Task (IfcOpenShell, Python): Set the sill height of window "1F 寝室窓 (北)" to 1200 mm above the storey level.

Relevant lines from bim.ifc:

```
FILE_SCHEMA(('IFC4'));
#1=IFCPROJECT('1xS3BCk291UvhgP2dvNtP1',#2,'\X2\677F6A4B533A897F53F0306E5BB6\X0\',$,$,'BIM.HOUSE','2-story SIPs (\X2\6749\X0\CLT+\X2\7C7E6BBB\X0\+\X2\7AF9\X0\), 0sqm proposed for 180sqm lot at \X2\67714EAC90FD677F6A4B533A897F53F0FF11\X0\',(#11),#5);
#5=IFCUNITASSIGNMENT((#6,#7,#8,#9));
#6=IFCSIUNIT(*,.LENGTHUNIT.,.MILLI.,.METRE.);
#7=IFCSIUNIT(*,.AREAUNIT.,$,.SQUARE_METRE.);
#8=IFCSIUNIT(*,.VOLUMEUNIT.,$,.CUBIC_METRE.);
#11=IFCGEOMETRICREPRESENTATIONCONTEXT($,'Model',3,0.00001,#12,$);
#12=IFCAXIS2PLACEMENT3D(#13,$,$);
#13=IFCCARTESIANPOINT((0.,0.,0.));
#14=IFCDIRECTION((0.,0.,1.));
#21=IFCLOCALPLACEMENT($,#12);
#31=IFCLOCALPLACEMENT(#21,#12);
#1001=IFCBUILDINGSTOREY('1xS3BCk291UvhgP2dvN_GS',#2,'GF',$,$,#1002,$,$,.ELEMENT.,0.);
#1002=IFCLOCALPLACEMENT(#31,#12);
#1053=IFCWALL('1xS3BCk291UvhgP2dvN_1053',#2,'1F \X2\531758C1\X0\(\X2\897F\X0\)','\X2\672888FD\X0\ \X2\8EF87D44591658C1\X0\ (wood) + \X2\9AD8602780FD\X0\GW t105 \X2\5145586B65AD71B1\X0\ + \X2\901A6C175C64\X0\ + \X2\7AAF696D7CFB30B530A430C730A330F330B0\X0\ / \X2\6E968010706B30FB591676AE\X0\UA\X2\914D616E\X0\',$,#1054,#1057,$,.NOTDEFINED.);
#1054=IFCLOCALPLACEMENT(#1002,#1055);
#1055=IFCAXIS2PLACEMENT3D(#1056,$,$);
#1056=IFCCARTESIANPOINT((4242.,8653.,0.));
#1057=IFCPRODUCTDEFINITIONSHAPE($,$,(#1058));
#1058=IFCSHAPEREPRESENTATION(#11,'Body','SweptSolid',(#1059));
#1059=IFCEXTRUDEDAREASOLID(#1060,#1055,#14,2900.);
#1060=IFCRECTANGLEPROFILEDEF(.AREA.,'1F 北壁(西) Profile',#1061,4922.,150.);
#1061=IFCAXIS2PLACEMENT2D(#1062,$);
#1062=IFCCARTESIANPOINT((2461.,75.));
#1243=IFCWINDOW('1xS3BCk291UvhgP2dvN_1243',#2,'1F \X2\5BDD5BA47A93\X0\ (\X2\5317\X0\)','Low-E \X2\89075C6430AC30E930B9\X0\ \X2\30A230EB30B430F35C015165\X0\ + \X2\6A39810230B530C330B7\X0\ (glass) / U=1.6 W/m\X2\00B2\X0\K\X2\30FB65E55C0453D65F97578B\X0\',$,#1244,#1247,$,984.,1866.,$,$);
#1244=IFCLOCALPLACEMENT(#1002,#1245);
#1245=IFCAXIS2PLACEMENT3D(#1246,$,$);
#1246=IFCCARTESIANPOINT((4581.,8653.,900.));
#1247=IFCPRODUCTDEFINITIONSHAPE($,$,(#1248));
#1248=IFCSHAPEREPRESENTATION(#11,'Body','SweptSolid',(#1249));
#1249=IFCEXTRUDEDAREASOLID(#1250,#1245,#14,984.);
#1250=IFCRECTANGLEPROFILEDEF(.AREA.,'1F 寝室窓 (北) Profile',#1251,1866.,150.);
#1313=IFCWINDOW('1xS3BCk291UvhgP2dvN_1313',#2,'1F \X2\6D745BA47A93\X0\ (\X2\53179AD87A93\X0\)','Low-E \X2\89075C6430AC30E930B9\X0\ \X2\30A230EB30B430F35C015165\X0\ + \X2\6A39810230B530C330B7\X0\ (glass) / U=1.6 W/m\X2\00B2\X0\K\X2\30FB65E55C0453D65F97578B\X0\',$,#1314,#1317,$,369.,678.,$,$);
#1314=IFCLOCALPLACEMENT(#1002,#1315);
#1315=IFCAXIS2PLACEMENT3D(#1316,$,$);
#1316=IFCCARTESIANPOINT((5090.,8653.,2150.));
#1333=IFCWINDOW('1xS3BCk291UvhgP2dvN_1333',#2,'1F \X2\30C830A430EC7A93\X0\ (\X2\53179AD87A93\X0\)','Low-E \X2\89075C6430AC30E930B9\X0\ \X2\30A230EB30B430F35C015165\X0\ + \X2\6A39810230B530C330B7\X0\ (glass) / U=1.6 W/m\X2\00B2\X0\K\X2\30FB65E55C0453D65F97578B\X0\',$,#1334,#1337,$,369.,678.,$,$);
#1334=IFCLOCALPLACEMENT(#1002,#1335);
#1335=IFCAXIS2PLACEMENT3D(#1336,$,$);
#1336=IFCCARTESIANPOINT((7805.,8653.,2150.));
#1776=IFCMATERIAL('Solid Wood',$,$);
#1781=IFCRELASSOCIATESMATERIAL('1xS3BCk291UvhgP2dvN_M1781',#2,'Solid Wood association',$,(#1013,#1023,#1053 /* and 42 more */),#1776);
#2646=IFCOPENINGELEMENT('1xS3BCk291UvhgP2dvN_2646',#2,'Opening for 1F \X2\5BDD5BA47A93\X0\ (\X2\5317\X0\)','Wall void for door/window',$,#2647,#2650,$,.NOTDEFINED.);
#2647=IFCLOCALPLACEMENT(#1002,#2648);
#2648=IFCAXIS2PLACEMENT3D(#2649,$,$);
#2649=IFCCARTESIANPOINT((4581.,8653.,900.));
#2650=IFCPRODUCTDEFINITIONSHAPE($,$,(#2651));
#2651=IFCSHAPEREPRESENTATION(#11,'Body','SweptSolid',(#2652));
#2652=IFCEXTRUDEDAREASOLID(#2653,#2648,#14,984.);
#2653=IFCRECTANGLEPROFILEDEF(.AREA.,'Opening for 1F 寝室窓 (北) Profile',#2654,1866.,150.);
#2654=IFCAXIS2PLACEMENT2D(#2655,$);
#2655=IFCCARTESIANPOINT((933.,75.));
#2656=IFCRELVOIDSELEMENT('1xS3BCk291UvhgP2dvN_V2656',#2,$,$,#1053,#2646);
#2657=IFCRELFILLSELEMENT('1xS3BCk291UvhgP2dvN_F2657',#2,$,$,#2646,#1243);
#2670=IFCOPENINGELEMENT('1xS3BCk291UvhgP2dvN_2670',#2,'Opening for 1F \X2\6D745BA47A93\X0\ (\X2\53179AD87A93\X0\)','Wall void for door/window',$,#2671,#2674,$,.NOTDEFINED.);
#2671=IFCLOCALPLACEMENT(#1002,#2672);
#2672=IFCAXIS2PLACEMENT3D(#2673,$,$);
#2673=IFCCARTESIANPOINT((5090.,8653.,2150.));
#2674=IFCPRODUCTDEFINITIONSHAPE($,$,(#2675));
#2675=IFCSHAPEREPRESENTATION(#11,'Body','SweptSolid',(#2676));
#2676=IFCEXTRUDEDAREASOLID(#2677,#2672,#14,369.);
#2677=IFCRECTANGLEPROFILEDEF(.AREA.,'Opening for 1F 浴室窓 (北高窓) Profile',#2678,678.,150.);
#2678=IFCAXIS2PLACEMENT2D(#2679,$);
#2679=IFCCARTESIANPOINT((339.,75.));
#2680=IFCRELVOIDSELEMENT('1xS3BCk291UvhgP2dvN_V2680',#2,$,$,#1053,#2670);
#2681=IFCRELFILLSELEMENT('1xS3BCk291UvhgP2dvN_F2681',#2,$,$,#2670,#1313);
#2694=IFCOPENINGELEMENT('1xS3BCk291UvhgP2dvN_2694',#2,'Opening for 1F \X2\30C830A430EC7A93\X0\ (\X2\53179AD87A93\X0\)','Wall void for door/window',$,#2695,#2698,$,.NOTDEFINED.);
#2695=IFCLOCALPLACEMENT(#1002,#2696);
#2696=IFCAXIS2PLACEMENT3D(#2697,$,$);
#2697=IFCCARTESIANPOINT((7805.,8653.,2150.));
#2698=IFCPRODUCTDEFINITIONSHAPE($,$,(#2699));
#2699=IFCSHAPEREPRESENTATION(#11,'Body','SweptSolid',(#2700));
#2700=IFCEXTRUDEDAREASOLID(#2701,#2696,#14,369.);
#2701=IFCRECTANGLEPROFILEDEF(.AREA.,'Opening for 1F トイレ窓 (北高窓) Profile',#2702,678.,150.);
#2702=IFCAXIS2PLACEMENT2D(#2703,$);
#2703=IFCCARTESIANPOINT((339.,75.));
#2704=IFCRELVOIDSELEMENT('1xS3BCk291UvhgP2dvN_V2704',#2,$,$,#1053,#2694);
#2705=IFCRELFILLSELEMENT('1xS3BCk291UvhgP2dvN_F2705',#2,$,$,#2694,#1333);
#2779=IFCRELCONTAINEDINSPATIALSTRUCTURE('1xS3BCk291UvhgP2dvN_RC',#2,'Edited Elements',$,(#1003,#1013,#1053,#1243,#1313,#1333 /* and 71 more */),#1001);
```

```python
import numpy as np
import ifcopenshell
import ifcopenshell.api.geometry
import ifcopenshell.geom
import ifcopenshell.util.element
import ifcopenshell.util.placement
import ifcopenshell.util.shape
import ifcopenshell.util.unit

model = ifcopenshell.open("bim.ifc")
unit_scale = ifcopenshell.util.unit.calculate_unit_scale(model)

window = model.by_guid("1xS3BCk291UvhgP2dvN_1243")
opening = window.FillsVoids[0].RelatingOpeningElement
storey = ifcopenshell.util.element.get_container(window, ifc_class="IfcBuildingStorey")
level = ifcopenshell.util.placement.get_local_placement(storey.ObjectPlacement)[2, 3]

# The opening's origin need not be at the sill, so measure its lowest point.
shape = ifcopenshell.geom.create_shape(ifcopenshell.geom.settings(), opening)
bottom = ifcopenshell.util.shape.get_shape_bottom_elevation(shape, shape.geometry) / unit_scale
dz = level + 1.2 / unit_scale - bottom

shift = np.array([0.0, 0.0, dz])
# The window is not placed relative to its opening, so move both.
for product in (opening, window):
    matrix = ifcopenshell.util.placement.get_local_placement(product.ObjectPlacement)
    matrix[:3, 3] += shift
    ifcopenshell.api.geometry.edit_object_placement(model, product=product, matrix=matrix, is_si=False)

print(f"moved by {dz * unit_scale:+.3f} m")

model.write("bim_updated.ifc")
```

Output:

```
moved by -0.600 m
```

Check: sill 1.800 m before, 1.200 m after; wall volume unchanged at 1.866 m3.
